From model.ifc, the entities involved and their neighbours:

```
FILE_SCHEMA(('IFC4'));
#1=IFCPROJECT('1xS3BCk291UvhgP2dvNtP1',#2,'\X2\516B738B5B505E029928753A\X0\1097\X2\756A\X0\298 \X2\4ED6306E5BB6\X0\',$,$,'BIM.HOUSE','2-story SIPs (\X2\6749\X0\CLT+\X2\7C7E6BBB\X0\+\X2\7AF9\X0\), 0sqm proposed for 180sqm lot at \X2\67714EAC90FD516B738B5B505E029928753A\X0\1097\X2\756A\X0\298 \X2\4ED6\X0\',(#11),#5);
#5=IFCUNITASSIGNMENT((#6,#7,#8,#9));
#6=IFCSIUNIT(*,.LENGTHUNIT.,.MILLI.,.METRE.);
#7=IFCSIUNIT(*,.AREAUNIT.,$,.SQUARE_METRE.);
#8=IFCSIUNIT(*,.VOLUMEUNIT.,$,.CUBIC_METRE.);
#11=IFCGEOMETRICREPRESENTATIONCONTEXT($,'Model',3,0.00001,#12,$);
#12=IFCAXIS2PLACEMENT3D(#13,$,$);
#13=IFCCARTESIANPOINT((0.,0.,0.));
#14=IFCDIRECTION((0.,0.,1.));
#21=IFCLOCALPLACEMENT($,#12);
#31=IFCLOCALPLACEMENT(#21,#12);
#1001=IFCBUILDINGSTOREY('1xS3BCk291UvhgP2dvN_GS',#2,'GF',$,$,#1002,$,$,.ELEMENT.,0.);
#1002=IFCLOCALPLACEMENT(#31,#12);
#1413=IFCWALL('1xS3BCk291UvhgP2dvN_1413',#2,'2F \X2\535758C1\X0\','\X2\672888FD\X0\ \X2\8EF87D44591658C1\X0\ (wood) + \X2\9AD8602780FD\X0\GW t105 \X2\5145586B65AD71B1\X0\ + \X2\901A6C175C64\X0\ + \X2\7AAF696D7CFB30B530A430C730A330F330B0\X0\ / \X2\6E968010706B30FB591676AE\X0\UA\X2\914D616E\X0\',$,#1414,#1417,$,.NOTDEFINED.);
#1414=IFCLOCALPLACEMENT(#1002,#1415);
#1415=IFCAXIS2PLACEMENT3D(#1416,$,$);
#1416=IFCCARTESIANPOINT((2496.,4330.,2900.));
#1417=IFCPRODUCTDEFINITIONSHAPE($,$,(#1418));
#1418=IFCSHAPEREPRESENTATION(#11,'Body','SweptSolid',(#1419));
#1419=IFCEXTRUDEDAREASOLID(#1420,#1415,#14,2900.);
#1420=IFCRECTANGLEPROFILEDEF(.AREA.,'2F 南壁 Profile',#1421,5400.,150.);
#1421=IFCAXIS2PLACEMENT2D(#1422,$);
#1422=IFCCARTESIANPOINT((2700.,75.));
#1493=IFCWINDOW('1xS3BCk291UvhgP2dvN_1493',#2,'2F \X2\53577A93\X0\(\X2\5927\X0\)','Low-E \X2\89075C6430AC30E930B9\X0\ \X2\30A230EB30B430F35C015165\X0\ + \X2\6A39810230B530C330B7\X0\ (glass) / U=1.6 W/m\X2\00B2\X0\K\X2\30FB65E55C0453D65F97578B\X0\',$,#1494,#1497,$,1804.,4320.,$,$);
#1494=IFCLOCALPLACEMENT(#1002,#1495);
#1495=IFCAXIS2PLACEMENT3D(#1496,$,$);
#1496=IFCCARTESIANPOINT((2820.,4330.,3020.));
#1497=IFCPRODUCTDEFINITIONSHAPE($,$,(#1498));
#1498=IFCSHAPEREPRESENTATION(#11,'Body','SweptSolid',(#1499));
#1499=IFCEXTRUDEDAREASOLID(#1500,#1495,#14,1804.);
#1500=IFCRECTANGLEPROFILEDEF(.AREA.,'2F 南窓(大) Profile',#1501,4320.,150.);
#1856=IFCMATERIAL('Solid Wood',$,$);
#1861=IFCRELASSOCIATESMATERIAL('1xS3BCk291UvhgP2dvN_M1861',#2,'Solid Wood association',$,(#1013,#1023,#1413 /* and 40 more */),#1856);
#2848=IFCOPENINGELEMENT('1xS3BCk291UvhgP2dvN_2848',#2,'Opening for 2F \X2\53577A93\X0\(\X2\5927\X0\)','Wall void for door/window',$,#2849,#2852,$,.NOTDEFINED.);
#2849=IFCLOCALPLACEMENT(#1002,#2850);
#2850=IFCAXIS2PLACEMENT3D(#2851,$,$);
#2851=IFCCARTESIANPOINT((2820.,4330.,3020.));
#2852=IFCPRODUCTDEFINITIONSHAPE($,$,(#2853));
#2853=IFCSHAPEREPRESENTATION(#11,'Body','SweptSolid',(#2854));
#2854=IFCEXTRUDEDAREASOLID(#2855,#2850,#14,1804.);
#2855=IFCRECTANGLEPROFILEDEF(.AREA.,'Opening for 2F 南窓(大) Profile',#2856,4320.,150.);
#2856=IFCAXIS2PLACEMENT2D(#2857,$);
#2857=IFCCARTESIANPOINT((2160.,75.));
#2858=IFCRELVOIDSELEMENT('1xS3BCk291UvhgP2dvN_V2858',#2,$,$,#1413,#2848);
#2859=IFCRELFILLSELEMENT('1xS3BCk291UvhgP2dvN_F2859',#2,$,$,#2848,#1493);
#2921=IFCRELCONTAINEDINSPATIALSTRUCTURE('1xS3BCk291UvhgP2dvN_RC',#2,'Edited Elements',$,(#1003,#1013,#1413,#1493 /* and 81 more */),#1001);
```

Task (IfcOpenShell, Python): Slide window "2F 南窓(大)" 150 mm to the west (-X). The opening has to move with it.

```python
import ifcopenshell
import ifcopenshell.api.geometry
import ifcopenshell.util.placement

model = ifcopenshell.open("model.ifc")

window = model.by_guid("1xS3BCk291UvhgP2dvN_1493")
opening = window.FillsVoids[0].RelatingOpeningElement
wall = opening.VoidsElements[0].RelatingBuildingElement

wall_matrix = ifcopenshell.util.placement.get_local_placement(wall.ObjectPlacement)
shift = wall_matrix[:3, 0] * -150.0
before = ifcopenshell.util.placement.get_local_placement(window.ObjectPlacement)[:3, 3].copy()

# The window is not placed relative to its opening, so move both.
for product in (opening, window):
    matrix = ifcopenshell.util.placement.get_local_placement(product.ObjectPlacement)
    matrix[:3, 3] += shift
    ifcopenshell.api.geometry.edit_object_placement(model, product=product, matrix=matrix, is_si=False)

after = ifcopenshell.util.placement.get_local_placement(window.ObjectPlacement)[:3, 3]
print("window moved by", (after - before).round(3) + 0.0)

model.write("model_edited.ifc")
```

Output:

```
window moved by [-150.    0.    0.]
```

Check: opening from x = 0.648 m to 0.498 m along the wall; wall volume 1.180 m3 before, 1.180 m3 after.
